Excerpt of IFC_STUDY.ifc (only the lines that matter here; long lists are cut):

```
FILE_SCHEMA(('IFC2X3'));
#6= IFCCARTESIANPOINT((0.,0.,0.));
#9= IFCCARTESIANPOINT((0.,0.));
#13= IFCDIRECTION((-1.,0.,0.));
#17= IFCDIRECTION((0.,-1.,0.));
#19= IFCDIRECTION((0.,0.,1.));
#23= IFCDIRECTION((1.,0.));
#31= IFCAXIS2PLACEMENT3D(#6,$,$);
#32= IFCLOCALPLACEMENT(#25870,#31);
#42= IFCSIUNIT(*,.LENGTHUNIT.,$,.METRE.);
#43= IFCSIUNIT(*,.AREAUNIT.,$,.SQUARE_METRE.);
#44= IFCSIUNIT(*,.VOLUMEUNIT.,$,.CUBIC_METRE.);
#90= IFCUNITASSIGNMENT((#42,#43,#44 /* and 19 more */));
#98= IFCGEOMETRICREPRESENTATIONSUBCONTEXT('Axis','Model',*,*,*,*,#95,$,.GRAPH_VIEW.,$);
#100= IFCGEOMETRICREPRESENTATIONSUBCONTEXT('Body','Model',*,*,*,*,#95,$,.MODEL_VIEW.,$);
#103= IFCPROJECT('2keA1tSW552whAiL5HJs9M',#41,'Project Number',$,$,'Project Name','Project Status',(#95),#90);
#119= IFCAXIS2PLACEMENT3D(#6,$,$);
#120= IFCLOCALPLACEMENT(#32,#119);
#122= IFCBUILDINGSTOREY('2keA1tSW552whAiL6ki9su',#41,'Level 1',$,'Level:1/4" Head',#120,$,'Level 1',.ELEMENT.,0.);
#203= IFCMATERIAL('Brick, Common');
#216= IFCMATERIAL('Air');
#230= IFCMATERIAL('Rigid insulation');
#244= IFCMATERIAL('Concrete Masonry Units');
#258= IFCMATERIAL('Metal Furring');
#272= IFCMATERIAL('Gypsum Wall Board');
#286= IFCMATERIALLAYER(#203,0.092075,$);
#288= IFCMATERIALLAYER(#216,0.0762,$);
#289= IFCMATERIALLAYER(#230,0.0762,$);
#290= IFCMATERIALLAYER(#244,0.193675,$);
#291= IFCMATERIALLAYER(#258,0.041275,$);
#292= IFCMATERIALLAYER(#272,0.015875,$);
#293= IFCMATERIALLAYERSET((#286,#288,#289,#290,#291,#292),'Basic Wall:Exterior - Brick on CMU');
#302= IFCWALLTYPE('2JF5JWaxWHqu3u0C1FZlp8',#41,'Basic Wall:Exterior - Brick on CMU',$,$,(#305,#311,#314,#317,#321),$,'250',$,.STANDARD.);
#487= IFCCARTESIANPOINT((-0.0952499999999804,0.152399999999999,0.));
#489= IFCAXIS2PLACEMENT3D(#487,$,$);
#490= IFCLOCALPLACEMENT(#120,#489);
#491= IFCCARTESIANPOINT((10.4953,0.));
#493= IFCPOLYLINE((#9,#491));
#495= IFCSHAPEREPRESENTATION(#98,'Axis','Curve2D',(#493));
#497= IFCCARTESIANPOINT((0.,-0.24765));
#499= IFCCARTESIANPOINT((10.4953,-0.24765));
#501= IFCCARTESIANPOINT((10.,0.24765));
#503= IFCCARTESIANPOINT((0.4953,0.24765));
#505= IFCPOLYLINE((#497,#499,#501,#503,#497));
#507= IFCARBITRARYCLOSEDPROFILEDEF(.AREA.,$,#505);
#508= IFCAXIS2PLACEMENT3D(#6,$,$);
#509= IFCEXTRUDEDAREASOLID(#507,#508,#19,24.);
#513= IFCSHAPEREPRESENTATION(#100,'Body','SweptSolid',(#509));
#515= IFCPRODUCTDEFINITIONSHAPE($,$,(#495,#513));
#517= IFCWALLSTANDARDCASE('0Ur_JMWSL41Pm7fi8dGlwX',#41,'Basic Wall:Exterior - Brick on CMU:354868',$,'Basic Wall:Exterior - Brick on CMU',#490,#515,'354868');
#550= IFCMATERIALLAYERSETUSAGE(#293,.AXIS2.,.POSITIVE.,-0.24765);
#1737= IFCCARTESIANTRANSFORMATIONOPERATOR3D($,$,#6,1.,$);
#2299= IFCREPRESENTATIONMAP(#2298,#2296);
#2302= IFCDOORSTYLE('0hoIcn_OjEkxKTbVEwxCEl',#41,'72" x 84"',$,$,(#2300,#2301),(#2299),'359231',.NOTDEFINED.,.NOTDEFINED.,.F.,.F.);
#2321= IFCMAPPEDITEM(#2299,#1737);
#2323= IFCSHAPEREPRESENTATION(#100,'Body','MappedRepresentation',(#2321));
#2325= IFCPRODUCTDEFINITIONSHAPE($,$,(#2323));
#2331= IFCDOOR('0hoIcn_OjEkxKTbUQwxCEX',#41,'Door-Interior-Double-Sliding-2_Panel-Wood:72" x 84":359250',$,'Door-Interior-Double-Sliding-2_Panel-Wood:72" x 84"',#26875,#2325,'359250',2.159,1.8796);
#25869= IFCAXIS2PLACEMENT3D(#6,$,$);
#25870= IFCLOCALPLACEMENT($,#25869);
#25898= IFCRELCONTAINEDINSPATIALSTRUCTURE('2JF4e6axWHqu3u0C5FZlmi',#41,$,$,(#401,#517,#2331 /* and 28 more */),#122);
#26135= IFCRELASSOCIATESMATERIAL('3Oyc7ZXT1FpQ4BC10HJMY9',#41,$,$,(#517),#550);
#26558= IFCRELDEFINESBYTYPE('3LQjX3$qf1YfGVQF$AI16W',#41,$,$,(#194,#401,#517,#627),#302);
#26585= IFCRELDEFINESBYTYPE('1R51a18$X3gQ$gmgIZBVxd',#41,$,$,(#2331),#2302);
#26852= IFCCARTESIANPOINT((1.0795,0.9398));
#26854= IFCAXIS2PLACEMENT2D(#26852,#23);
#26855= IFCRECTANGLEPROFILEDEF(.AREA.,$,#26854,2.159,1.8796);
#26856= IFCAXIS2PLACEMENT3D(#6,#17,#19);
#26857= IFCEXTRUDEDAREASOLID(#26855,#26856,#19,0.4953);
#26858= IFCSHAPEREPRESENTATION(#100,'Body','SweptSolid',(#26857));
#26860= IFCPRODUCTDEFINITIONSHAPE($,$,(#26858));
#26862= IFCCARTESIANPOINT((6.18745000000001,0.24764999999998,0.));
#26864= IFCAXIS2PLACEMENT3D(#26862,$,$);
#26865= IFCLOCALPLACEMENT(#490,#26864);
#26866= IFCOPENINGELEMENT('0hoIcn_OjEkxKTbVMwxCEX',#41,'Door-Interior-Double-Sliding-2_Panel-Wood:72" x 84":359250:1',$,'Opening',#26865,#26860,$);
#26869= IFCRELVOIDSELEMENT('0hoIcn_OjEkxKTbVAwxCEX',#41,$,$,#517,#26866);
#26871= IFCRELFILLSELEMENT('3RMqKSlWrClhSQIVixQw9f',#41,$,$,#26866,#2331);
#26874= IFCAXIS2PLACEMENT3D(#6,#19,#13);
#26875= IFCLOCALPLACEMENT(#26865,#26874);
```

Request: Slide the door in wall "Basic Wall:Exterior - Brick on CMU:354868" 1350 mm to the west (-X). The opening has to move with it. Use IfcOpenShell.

```python
import ifcopenshell
import ifcopenshell.api.geometry
import ifcopenshell.util.placement

model = ifcopenshell.open("IFC_STUDY.ifc")

door = model.by_guid("0hoIcn_OjEkxKTbUQwxCEX")
opening = door.FillsVoids[0].RelatingOpeningElement
wall = opening.VoidsElements[0].RelatingBuildingElement

wall_matrix = ifcopenshell.util.placement.get_local_placement(wall.ObjectPlacement)
shift = wall_matrix[:3, 0] * -1.35
before = ifcopenshell.util.placement.get_local_placement(door.ObjectPlacement)[:3, 3].copy()

# The door is placed relative to its opening, so it follows when the opening moves.
matrix = ifcopenshell.util.placement.get_local_placement(opening.ObjectPlacement)
matrix[:3, 3] += shift
ifcopenshell.api.geometry.edit_object_placement(
    model, product=opening, matrix=matrix, is_si=False, should_transform_children=True
)

after = ifcopenshell.util.placement.get_local_placement(door.ObjectPlacement)[:3, 3]
print("door moved by", (after - before).round(3) + 0.0)

model.write("IFC_STUDY_updated.ifc")
```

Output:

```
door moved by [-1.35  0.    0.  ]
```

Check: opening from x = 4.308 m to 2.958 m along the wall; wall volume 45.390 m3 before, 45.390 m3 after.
